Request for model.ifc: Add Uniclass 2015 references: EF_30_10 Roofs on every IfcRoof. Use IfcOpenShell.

First a look at what the model holds.

```python
import ifcopenshell

model = ifcopenshell.open("model.ifc")
print(model.schema)
print("classifications:", [c.Name for c in model.by_type("IfcClassification")])
for ifc_class in ("IfcDoor", "IfcRoof", "IfcStair", "IfcWall", "IfcWindow"):
    print(ifc_class, len(model.by_type(ifc_class)))
```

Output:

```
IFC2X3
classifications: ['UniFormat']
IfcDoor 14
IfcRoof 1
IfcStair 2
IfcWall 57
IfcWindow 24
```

```python
import ifcopenshell
import ifcopenshell.api.classification

model = ifcopenshell.open("model.ifc")

# IFC2X3 requires Source and Edition and has no link from the project to the system.
system = model.create_entity("IfcClassification", Source="NBS", Edition="2015", Name="Uniclass 2015")

codes = {
    "IfcRoof": ("EF_30_10", "Roofs"),
}
for ifc_class, (code, name) in codes.items():
    products = model.by_type(ifc_class)
    ifcopenshell.api.classification.add_reference(
        model, products=products, classification=system, identification=code, name=name
    )
    print(code, len(products))

model.write("model_rev.ifc")
```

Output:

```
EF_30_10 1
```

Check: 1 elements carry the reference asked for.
